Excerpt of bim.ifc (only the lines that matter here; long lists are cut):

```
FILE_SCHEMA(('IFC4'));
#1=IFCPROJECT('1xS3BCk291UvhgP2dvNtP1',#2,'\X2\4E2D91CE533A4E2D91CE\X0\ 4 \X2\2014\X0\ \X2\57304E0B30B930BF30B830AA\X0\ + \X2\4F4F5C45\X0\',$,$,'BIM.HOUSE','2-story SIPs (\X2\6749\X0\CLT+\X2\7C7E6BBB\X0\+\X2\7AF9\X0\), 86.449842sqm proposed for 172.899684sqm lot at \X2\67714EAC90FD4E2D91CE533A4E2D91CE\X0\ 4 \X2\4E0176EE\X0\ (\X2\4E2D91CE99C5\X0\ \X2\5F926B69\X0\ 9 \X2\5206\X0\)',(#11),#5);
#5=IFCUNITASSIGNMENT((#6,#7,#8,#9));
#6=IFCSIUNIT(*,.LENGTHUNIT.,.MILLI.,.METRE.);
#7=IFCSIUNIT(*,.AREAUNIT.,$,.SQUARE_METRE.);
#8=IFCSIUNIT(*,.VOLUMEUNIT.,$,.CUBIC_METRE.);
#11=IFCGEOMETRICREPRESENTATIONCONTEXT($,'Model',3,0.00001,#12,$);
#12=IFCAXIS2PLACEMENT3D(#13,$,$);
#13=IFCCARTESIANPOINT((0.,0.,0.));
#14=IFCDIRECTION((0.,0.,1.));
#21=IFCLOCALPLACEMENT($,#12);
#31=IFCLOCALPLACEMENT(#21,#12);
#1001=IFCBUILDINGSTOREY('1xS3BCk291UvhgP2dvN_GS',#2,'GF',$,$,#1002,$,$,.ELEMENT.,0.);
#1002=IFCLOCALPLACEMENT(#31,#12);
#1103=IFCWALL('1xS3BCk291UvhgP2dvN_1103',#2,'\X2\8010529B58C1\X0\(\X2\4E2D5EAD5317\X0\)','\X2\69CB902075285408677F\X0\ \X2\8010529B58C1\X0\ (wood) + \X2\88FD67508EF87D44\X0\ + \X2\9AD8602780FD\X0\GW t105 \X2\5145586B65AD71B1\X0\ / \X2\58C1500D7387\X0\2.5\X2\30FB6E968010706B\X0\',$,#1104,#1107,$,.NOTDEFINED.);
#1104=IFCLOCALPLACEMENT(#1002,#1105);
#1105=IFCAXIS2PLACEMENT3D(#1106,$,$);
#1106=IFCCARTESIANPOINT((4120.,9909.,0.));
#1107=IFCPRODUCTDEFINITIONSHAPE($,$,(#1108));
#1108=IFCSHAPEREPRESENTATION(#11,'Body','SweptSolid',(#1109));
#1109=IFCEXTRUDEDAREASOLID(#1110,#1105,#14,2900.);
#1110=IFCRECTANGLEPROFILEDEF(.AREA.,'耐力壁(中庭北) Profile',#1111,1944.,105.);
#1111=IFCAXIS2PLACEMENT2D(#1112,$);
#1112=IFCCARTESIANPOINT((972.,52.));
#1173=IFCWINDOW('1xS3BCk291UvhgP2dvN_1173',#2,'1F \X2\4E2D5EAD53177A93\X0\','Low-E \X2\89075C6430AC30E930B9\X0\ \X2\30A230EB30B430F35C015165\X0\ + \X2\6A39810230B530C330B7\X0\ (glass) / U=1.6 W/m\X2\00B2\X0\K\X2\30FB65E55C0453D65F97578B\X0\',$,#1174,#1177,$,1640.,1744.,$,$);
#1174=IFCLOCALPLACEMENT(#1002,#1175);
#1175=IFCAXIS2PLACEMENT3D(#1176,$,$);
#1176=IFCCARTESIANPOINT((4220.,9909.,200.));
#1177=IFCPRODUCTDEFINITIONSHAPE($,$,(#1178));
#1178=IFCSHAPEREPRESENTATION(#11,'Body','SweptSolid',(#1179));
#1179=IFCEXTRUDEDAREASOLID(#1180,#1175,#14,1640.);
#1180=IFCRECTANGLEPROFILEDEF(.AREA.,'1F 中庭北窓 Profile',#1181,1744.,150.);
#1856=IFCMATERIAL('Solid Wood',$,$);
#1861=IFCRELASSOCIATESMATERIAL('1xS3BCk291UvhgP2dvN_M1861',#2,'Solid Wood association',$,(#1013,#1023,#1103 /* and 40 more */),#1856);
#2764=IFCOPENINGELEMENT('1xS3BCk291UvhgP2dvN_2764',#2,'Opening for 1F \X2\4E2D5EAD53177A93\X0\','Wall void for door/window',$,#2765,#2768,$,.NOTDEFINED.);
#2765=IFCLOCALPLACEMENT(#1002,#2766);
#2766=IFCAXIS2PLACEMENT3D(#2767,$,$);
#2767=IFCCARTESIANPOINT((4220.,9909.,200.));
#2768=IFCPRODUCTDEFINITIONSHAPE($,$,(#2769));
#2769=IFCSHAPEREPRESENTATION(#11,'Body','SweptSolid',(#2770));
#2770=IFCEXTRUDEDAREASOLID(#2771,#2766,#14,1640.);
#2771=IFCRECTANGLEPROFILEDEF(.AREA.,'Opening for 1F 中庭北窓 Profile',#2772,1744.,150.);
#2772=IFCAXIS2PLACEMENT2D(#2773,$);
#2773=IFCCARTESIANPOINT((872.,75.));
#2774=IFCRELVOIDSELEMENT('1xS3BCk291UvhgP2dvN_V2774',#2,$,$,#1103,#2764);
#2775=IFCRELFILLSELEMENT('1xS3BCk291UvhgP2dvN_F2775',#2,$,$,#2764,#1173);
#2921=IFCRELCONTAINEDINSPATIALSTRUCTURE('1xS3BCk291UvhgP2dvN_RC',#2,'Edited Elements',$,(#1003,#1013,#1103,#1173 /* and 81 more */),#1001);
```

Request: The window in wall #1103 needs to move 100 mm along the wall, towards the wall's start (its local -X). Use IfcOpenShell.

```python
import ifcopenshell
import ifcopenshell.api.geometry
import ifcopenshell.util.placement
import ifcopenshell.util.unit

model = ifcopenshell.open("bim.ifc")
unit_scale = ifcopenshell.util.unit.calculate_unit_scale(model)

window = model.by_id(1173)
opening = window.FillsVoids[0].RelatingOpeningElement
wall = opening.VoidsElements[0].RelatingBuildingElement

wall_matrix = ifcopenshell.util.placement.get_local_placement(wall.ObjectPlacement)
shift = wall_matrix[:3, 0] * -0.1 / unit_scale
before = ifcopenshell.util.placement.get_local_placement(window.ObjectPlacement)[:3, 3].copy()

# The window is not placed relative to its opening, so move both.
for product in (opening, window):
    matrix = ifcopenshell.util.placement.get_local_placement(product.ObjectPlacement)
    matrix[:3, 3] += shift
    ifcopenshell.api.geometry.edit_object_placement(model, product=product, matrix=matrix, is_si=False)

after = ifcopenshell.util.placement.get_local_placement(window.ObjectPlacement)[:3, 3]
print("window moved by", (after - before).round(3) + 0.0)

model.write("bim-out.ifc")
```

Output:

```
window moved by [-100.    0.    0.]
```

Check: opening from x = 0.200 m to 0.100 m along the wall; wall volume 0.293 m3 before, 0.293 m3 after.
